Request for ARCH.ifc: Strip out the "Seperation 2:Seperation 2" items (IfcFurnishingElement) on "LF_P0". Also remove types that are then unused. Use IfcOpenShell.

First a look at what the model holds.

```python
import ifcopenshell
import ifcopenshell.util.element

model = ifcopenshell.open("ARCH.ifc")
print(model.schema)
storey = next(s for s in model.by_type("IfcBuildingStorey") if s.Name == "LF_P0")
furniture = [e for e in ifcopenshell.util.element.get_decomposition(storey) if e.is_a("IfcFurnishingElement")]
seen = {}
for e in furniture:
    element_type = ifcopenshell.util.element.get_type(e)
    name = element_type.Name if element_type not in (None, e) else None
    seen[name] = seen.get(name, 0) + 1
for name, count in sorted(seen.items(), key=str):
    print(count, "x", name)
```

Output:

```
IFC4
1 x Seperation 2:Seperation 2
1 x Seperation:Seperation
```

```python
import ifcopenshell
import ifcopenshell.api.root
import ifcopenshell.util.element

model = ifcopenshell.open("ARCH.ifc")

storey = next(s for s in model.by_type("IfcBuildingStorey") if s.Name == "LF_P0")
furniture = [e for e in ifcopenshell.util.element.get_decomposition(storey) if e.is_a("IfcFurnishingElement")]
targets = [e for e in furniture if (t := ifcopenshell.util.element.get_type(e)) not in (None, e) and t.Name == "Seperation 2:Seperation 2"]
types = {ifcopenshell.util.element.get_type(e) for e in targets} - {None, *targets}

for e in targets:
    ifcopenshell.api.root.remove_product(model, product=e)
print(len(targets), "removed")

unused = [t for t in types if not ifcopenshell.util.element.get_types(t)]
for t in unused:
    ifcopenshell.api.root.remove_product(model, product=t)
print(len(unused), "unused types removed")

model.write("ARCH_updated.ifc")
```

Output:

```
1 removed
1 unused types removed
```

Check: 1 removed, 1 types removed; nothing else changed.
